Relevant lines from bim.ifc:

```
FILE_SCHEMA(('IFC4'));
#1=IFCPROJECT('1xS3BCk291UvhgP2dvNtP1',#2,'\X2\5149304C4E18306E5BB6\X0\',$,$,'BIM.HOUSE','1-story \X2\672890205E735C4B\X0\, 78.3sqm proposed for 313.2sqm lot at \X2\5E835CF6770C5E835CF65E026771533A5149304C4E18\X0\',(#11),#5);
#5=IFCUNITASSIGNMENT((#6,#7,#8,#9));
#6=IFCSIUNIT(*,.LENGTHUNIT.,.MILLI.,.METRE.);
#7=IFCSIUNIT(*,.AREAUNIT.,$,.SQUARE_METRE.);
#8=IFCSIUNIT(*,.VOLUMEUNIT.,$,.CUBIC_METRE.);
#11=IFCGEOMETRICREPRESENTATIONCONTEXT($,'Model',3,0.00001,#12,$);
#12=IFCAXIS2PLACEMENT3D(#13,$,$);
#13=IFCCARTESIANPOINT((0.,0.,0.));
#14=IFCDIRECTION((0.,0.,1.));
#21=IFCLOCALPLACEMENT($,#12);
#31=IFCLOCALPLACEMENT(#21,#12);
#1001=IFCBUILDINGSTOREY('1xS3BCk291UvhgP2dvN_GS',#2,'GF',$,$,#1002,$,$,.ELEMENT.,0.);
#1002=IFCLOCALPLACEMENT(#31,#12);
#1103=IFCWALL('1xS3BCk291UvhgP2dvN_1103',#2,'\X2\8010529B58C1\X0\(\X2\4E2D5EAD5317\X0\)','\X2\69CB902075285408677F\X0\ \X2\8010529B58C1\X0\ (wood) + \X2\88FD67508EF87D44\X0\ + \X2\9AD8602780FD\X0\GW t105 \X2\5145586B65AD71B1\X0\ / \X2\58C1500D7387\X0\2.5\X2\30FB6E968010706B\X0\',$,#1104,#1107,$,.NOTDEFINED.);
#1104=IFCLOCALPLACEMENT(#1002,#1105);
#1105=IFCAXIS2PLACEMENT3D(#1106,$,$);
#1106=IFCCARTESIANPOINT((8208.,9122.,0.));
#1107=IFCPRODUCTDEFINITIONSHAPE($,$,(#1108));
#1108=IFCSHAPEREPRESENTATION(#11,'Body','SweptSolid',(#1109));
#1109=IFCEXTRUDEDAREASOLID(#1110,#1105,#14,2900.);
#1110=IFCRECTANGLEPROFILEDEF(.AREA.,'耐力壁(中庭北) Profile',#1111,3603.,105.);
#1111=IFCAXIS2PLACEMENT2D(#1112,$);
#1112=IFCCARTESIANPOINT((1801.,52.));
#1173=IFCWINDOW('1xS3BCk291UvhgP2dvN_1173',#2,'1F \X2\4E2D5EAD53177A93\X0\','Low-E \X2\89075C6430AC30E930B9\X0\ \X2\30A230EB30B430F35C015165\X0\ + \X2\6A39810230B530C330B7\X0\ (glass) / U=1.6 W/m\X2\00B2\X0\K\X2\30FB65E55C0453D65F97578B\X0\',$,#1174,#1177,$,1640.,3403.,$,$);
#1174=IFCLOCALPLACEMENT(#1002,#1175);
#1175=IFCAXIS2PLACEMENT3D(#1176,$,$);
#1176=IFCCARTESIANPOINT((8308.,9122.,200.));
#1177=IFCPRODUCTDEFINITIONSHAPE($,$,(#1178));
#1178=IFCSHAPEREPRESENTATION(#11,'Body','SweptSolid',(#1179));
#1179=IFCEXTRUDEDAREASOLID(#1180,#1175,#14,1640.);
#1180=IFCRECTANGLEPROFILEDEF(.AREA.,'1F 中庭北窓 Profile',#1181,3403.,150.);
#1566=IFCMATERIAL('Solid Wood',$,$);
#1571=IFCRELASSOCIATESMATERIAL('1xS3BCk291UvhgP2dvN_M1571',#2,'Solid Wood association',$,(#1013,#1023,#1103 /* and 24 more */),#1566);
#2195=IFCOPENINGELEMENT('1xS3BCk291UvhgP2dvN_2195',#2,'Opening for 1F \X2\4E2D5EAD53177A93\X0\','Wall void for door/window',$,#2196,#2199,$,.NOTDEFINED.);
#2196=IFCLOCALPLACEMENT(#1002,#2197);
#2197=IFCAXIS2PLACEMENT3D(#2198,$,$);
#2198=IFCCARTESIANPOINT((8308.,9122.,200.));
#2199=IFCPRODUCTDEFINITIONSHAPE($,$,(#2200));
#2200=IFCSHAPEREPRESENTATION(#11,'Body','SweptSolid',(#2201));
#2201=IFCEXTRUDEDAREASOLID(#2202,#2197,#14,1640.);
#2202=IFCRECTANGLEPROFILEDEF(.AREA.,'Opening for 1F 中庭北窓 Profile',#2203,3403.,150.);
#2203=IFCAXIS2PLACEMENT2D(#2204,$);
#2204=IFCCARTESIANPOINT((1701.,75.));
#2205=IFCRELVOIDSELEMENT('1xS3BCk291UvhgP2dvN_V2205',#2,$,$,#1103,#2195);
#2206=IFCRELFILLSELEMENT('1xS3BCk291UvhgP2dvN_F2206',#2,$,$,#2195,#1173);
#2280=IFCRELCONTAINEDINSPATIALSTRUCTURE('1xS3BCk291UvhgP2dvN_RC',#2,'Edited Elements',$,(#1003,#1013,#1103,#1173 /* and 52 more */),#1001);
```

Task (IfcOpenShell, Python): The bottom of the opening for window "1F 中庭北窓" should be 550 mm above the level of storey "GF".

```python
import numpy as np
import ifcopenshell
import ifcopenshell.api.geometry
import ifcopenshell.geom
import ifcopenshell.util.element
import ifcopenshell.util.placement
import ifcopenshell.util.shape
import ifcopenshell.util.unit

model = ifcopenshell.open("bim.ifc")
unit_scale = ifcopenshell.util.unit.calculate_unit_scale(model)

window = model.by_guid("1xS3BCk291UvhgP2dvN_1173")
opening = window.FillsVoids[0].RelatingOpeningElement
storey = ifcopenshell.util.element.get_container(window, ifc_class="IfcBuildingStorey")
level = ifcopenshell.util.placement.get_local_placement(storey.ObjectPlacement)[2, 3]

# The opening's origin need not be at the sill, so measure its lowest point.
shape = ifcopenshell.geom.create_shape(ifcopenshell.geom.settings(), opening)
bottom = ifcopenshell.util.shape.get_shape_bottom_elevation(shape, shape.geometry) / unit_scale
dz = level + 0.55 / unit_scale - bottom

shift = np.array([0.0, 0.0, dz])
# The window is not placed relative to its opening, so move both.
for product in (opening, window):
    matrix = ifcopenshell.util.placement.get_local_placement(product.ObjectPlacement)
    matrix[:3, 3] += shift
    ifcopenshell.api.geometry.edit_object_placement(model, product=product, matrix=matrix, is_si=False)

print(f"moved by {dz * unit_scale:+.3f} m")

model.write("bim_edited.ifc")
```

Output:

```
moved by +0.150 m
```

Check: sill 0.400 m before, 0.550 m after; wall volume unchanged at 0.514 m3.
